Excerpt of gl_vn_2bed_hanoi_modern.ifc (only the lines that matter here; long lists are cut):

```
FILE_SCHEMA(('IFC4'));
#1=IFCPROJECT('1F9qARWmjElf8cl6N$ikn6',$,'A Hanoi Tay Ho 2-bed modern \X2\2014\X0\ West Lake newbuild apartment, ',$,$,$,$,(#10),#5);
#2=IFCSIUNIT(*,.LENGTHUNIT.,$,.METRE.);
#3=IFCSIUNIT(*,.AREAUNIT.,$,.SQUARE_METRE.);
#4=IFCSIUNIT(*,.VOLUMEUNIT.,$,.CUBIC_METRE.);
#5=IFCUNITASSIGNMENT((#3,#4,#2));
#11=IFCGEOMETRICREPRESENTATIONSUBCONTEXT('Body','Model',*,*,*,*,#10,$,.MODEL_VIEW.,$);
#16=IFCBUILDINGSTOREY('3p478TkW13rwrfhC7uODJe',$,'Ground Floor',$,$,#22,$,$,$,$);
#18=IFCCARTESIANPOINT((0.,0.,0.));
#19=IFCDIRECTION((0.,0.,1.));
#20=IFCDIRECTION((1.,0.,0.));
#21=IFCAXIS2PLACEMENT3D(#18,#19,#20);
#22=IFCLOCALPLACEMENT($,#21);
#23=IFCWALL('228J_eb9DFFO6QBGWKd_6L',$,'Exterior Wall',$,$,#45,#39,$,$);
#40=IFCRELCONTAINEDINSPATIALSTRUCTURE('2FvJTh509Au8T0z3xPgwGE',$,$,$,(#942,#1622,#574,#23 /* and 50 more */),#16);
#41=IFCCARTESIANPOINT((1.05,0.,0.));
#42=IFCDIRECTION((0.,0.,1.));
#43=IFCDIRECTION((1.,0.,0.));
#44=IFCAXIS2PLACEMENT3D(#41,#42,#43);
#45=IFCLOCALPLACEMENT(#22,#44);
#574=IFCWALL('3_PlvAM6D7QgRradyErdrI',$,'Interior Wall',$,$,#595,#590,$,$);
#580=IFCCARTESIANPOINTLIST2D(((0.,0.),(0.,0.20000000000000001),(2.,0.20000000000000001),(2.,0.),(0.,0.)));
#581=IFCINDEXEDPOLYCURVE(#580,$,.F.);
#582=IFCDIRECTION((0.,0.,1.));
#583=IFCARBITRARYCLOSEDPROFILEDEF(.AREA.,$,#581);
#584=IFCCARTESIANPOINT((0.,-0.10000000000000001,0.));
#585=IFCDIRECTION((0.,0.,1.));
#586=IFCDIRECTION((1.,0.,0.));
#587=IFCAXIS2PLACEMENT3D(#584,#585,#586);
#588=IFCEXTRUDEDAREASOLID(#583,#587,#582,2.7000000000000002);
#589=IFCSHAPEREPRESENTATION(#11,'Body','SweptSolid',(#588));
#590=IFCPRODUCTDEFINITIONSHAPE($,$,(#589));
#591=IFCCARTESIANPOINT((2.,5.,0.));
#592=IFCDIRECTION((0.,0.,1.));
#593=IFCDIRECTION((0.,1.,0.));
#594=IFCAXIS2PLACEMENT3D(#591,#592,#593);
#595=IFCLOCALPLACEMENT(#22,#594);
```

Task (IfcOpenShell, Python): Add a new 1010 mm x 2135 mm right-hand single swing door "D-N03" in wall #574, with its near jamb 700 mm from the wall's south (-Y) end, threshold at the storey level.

```python
import numpy as np
import ifcopenshell
import ifcopenshell.api.feature
import ifcopenshell.api.geometry
import ifcopenshell.api.root
import ifcopenshell.api.spatial
import ifcopenshell.geom
import ifcopenshell.util.element
import ifcopenshell.util.placement
import ifcopenshell.util.representation
import ifcopenshell.util.shape
import ifcopenshell.util.unit

model = ifcopenshell.open("gl_vn_2bed_hanoi_modern.ifc")
unit_scale = ifcopenshell.util.unit.calculate_unit_scale(model)
settings = ifcopenshell.geom.settings()


def volume(element):
    """Net volume in cubic metres, openings subtracted."""
    shape = ifcopenshell.geom.create_shape(settings, element)
    return ifcopenshell.util.shape.get_volume(shape.geometry)


wall = model.by_guid("3_PlvAM6D7QgRradyErdrI")
storey = ifcopenshell.util.element.get_container(wall, ifc_class="IfcBuildingStorey")
context = ifcopenshell.util.representation.get_context(model, "Model", "Body", "MODEL_VIEW")
before = volume(wall)

width, height, from_end, sill = 1.01, 2.135, 0.7, 0.0  # metres

# The wall runs along its own X axis, and the end named is its -X end.
wall_shape = ifcopenshell.geom.create_shape(settings, wall)
x, y, z = ifcopenshell.util.shape.get_vertices(wall_shape.geometry).T
start = x.min() + from_end
face, thickness = float(y.min()), float(y.max() - y.min())
wall_matrix = ifcopenshell.util.placement.get_local_placement(wall.ObjectPlacement)
level = ifcopenshell.util.placement.get_local_placement(storey.ObjectPlacement)[2, 3]


def in_wall(x, y):
    """Placement at x, y metres in the wall's axes, at sill height."""
    matrix = wall_matrix.copy()
    matrix[:, 3] = wall_matrix @ np.array([x / unit_scale, y / unit_scale, 0.0, 1.0])
    matrix[2, 3] = level + sill / unit_scale
    return matrix


# Opening: a box that overshoots both wall faces by 50 mm.
opening = ifcopenshell.api.root.create_entity(model, ifc_class="IfcOpeningElement", predefined_type="OPENING")
box = ifcopenshell.api.geometry.add_wall_representation(
    model, context=context, length=width, height=height, thickness=thickness + 0.1
)
ifcopenshell.api.geometry.assign_representation(model, product=opening, representation=box)
ifcopenshell.api.geometry.edit_object_placement(model, product=opening, matrix=in_wall(start, face - 0.05), is_si=False)
ifcopenshell.api.feature.add_feature(model, feature=opening, element=wall)

door = ifcopenshell.api.root.create_entity(model, ifc_class="IfcDoor", name="D-N03", predefined_type="DOOR")
door.OverallWidth, door.OverallHeight = width / unit_scale, height / unit_scale
door.OperationType = "SINGLE_SWING_RIGHT"
body = ifcopenshell.api.geometry.add_door_representation(
    model,
    context=context,
    overall_width=door.OverallWidth,
    overall_height=door.OverallHeight,
    operation_type="SINGLE_SWING_RIGHT",
    lining_properties={"LiningDepth": thickness / unit_scale, "ThresholdDepth": thickness / unit_scale},
)
ifcopenshell.api.geometry.assign_representation(model, product=door, representation=body)
ifcopenshell.api.spatial.assign_container(model, products=[door], relating_structure=storey)
ifcopenshell.api.feature.add_filling(model, opening=opening, element=door)

# The lining spans the wall, so the door starts at the wall face.
ifcopenshell.api.geometry.edit_object_placement(model, product=door, matrix=in_wall(start, face), is_si=False)

after = volume(wall)

print(f"wall volume {before:.3f} -> {after:.3f} m3")

model.write("gl_vn_2bed_hanoi_modern_rev.ifc")
```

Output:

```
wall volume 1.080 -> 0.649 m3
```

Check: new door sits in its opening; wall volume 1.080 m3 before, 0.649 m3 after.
